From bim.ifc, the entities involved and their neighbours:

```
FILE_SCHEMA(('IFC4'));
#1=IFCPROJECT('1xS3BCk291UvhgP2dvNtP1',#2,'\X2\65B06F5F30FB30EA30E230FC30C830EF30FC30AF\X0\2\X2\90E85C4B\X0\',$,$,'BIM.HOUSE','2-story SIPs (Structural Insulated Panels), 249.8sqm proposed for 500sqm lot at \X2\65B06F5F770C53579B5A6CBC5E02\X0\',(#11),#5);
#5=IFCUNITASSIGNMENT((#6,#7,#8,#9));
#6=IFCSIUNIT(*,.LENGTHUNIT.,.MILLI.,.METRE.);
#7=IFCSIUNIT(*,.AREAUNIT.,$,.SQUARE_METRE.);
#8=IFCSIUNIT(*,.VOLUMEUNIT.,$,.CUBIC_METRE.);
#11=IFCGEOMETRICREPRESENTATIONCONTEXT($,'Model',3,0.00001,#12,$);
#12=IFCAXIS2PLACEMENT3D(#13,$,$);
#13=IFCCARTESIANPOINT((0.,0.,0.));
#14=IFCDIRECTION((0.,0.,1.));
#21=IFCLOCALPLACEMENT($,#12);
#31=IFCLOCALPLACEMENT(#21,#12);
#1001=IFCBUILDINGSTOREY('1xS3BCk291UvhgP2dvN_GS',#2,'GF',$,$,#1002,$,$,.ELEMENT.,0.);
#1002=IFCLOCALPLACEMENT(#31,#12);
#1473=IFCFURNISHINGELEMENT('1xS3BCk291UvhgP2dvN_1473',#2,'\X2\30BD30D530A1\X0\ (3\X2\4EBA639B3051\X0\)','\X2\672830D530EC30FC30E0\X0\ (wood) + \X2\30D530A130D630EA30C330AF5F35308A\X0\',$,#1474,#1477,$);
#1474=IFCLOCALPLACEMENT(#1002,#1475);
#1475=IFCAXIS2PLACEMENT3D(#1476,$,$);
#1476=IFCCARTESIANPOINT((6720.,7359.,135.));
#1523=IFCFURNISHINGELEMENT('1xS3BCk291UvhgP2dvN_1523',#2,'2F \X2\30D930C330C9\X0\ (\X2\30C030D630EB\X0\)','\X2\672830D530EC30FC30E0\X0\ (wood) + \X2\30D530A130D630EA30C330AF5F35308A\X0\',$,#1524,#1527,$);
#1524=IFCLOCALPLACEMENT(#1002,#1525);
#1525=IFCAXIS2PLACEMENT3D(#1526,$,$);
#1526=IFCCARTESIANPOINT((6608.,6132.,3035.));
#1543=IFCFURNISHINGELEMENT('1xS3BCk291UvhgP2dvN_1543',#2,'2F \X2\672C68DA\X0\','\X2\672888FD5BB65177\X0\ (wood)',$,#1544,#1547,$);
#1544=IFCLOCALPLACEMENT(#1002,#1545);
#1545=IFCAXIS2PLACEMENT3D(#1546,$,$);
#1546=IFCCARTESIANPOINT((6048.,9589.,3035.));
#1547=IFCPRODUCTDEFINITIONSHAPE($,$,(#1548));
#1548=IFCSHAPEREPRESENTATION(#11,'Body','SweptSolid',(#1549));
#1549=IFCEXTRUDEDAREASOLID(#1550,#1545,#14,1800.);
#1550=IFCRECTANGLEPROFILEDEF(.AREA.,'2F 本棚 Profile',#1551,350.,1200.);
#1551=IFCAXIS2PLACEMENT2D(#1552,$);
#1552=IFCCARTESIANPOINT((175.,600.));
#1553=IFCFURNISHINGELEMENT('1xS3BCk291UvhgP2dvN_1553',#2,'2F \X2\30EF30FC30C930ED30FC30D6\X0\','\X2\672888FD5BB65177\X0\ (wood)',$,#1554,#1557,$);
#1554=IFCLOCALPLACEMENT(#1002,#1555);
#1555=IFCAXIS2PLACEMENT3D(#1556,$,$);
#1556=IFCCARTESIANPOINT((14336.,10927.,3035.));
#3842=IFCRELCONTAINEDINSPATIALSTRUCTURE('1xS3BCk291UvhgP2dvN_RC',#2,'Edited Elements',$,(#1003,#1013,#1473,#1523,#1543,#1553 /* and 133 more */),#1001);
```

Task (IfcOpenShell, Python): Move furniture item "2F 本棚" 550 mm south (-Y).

```python
import ifcopenshell
import ifcopenshell.api.geometry
import ifcopenshell.util.placement
import ifcopenshell.util.unit

model = ifcopenshell.open("bim.ifc")
unit_scale = ifcopenshell.util.unit.calculate_unit_scale(model)

item = model.by_guid("1xS3BCk291UvhgP2dvN_1543")
matrix = ifcopenshell.util.placement.get_local_placement(item.ObjectPlacement)
matrix[1, 3] -= 0.55 / unit_scale
ifcopenshell.api.geometry.edit_object_placement(model, product=item, matrix=matrix, is_si=False)

print(ifcopenshell.util.placement.get_local_placement(item.ObjectPlacement).round(3) + 0.0)

model.write("bim_rev.ifc")
```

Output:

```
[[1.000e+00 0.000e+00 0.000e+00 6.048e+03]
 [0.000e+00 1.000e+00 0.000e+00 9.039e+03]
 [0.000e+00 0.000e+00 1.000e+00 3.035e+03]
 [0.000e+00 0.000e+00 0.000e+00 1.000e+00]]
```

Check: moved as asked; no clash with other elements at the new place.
